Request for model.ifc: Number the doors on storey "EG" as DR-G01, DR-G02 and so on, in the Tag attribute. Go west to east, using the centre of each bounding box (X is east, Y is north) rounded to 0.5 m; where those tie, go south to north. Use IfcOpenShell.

First a look at what the model holds.

```python
import ifcopenshell
import ifcopenshell.util.element
import ifcopenshell.util.placement

model = ifcopenshell.open("model.ifc")
print(model.schema)
storey = next(s for s in model.by_type("IfcBuildingStorey") if s.Name == "EG")
doors = [e for e in ifcopenshell.util.element.get_decomposition(storey) if e.is_a("IfcDoor")]
for e in sorted(doors, key=lambda e: e.id()):
    origin = ifcopenshell.util.placement.get_local_placement(e.ObjectPlacement)[:3, 3]
    print(e.id(), e.Tag, e.Name, origin.round(2) + 0.0, sep=" | ")
```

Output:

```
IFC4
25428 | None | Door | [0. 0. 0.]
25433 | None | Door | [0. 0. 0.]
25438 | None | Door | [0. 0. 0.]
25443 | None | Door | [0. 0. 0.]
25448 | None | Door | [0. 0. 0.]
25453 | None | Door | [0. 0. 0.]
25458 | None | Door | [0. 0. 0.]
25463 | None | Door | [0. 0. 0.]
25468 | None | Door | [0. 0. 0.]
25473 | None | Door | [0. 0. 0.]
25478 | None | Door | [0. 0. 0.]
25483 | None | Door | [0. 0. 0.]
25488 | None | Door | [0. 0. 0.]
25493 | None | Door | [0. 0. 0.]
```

```python
import ifcopenshell
import ifcopenshell.geom
import ifcopenshell.util.element
import ifcopenshell.util.shape

model = ifcopenshell.open("model.ifc")
settings = ifcopenshell.geom.settings()
settings.set("use-world-coords", True)


def centre(element):
    shape = ifcopenshell.geom.create_shape(settings, element)
    return ifcopenshell.util.shape.get_bbox_centroid(shape.geometry)


storey = next(s for s in model.by_type("IfcBuildingStorey") if s.Name == "EG")
doors = [e for e in ifcopenshell.util.element.get_decomposition(storey) if e.is_a("IfcDoor")]

# Insertion points can sit at a corner or the storey origin, so sort by the geometry (in metres).
centres = {e: centre(e) for e in doors}
doors.sort(key=lambda e: (round(centres[e][0] / 0.5), centres[e][1]))

for i, e in enumerate(doors, start=1):
    number = f"DR-G{i:02d}"
    e.Tag = number
    print(e.id(), number)

model.write("model-out.ifc")
```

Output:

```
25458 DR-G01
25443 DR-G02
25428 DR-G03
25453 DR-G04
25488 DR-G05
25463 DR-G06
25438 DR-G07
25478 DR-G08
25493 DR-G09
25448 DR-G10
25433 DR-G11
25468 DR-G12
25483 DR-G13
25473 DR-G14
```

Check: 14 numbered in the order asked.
